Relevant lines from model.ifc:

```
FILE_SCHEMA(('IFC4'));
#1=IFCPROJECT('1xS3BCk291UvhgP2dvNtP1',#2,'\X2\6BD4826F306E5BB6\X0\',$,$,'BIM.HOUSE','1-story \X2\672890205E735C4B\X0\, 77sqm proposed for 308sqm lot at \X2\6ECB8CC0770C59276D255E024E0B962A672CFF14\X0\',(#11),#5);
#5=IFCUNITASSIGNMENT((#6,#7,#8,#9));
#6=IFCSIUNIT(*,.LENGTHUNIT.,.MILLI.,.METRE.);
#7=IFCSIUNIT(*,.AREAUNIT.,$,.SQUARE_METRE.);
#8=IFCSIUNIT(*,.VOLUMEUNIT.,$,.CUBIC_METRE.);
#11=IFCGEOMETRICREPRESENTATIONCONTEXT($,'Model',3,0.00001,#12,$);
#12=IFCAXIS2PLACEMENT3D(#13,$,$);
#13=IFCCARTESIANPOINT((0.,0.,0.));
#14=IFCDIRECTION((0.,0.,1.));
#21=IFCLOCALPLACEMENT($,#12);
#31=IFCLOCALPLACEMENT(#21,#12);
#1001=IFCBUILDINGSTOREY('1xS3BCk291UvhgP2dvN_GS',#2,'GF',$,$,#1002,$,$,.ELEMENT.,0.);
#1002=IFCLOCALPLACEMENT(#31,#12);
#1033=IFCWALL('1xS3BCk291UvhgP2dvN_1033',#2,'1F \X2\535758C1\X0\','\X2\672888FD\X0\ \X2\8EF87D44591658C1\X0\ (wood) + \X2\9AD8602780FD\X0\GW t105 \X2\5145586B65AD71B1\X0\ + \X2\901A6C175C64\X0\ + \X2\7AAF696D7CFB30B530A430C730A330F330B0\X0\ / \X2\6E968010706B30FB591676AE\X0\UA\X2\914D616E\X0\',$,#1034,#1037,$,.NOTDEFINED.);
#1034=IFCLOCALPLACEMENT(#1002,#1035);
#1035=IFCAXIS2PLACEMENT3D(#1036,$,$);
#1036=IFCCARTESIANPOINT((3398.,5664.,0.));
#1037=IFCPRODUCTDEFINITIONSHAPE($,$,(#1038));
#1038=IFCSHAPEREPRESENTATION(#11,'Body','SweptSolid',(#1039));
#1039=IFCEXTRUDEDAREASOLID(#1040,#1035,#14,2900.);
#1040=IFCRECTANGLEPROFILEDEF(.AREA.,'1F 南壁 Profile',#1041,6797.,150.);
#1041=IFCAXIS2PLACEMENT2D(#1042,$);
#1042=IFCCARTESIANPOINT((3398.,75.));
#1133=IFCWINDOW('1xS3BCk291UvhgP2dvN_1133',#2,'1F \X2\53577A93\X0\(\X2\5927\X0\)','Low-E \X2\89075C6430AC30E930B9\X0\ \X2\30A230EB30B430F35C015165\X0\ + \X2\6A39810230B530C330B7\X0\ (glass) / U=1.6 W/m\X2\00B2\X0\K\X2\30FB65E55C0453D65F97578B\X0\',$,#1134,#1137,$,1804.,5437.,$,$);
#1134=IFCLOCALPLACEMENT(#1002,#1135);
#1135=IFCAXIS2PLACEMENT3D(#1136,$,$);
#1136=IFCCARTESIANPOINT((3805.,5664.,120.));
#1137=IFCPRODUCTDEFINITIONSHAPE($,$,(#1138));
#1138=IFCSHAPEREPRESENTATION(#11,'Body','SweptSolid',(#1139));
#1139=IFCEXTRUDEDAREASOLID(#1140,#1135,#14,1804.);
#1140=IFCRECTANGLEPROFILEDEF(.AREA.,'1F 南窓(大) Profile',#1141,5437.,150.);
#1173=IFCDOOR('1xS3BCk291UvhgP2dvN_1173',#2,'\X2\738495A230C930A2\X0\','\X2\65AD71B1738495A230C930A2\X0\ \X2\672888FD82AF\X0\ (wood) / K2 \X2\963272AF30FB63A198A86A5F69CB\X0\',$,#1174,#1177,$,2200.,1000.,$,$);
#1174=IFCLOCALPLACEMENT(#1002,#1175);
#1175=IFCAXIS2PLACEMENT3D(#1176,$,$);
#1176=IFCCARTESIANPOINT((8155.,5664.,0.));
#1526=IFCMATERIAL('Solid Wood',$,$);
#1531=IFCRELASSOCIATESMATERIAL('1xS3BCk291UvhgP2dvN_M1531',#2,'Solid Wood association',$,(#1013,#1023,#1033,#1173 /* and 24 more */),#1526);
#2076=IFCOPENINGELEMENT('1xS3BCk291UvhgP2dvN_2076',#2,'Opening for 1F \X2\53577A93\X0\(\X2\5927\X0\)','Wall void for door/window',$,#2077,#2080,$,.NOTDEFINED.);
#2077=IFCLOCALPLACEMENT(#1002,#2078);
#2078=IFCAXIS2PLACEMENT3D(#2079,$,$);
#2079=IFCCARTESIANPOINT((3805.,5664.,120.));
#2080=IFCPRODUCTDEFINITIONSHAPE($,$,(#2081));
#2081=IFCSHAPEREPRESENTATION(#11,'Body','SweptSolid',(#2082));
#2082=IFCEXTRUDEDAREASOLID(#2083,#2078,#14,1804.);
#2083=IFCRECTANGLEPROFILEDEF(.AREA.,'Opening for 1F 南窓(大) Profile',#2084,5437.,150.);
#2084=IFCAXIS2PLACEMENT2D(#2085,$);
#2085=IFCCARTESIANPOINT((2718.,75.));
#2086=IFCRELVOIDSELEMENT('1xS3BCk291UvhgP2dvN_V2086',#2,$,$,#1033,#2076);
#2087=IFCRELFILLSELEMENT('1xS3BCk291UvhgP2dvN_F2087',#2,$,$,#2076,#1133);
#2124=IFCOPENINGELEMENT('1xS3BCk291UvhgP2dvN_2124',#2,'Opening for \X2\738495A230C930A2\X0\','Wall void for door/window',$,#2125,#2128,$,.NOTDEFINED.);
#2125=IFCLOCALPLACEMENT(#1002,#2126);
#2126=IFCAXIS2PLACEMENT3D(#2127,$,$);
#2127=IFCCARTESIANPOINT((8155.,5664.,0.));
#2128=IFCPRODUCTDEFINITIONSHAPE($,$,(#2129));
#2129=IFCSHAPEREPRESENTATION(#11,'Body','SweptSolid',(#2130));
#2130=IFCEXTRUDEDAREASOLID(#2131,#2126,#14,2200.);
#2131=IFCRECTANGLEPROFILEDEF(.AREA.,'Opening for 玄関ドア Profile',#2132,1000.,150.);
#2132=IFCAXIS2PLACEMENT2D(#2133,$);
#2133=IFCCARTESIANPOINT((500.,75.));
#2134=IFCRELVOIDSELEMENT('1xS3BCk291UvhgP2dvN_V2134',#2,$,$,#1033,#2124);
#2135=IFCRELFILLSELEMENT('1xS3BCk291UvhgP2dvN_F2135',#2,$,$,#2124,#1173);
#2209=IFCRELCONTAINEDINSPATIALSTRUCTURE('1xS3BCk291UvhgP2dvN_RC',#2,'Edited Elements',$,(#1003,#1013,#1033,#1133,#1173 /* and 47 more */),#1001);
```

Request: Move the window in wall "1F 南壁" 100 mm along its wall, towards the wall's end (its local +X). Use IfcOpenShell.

```python
import ifcopenshell
import ifcopenshell.api.geometry
import ifcopenshell.util.placement
import ifcopenshell.util.unit

model = ifcopenshell.open("model.ifc")
unit_scale = ifcopenshell.util.unit.calculate_unit_scale(model)

window = model.by_guid("1xS3BCk291UvhgP2dvN_1133")
opening = window.FillsVoids[0].RelatingOpeningElement
wall = opening.VoidsElements[0].RelatingBuildingElement

wall_matrix = ifcopenshell.util.placement.get_local_placement(wall.ObjectPlacement)
shift = wall_matrix[:3, 0] * 0.1 / unit_scale
before = ifcopenshell.util.placement.get_local_placement(window.ObjectPlacement)[:3, 3].copy()

# The window is not placed relative to its opening, so move both.
for product in (opening, window):
    matrix = ifcopenshell.util.placement.get_local_placement(product.ObjectPlacement)
    matrix[:3, 3] += shift
    ifcopenshell.api.geometry.edit_object_placement(model, product=product, matrix=matrix, is_si=False)

after = ifcopenshell.util.placement.get_local_placement(window.ObjectPlacement)[:3, 3]
print("window moved by", (after - before).round(3) + 0.0)

model.write("model_updated.ifc")
```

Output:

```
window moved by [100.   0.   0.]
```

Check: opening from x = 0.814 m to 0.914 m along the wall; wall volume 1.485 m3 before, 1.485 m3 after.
